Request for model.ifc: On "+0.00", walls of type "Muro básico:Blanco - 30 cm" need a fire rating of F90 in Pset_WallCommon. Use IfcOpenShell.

First a look at what the model holds.

```python
import ifcopenshell
import ifcopenshell.util.element

model = ifcopenshell.open("model.ifc")
print(model.schema)
storey = next(s for s in model.by_type("IfcBuildingStorey") if s.Name == "+0.00")
walls = [e for e in ifcopenshell.util.element.get_decomposition(storey) if e.is_a("IfcWall")]
seen = {}
for e in walls:
    element_type = ifcopenshell.util.element.get_type(e)
    key = (element_type.Name if element_type != e and element_type else None, ifcopenshell.util.element.get_pset(e, "Pset_WallCommon", "FireRating"))
    seen[key] = seen.get(key, 0) + 1
for (name, value), count in sorted(seen.items(), key=str):
    print(count, "x", name, "|", value)
```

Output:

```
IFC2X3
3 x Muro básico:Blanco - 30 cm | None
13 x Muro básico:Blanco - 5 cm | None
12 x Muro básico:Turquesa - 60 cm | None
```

```python
import ifcopenshell
import ifcopenshell.api.pset
import ifcopenshell.util.element

model = ifcopenshell.open("model.ifc")

storey = next(s for s in model.by_type("IfcBuildingStorey") if s.Name == "+0.00")
walls = [e for e in ifcopenshell.util.element.get_decomposition(storey) if e.is_a("IfcWall")]

count = 0
for e in walls:
    element_type = ifcopenshell.util.element.get_type(e)
    if element_type in (None, e) or element_type.Name != "Muro básico:Blanco - 30 cm":
        continue
    # add_pset returns the element's existing set when there is one.
    pset = ifcopenshell.api.pset.add_pset(model, product=e, name="Pset_WallCommon")
    ifcopenshell.api.pset.edit_pset(model, pset=pset, properties={"FireRating": "F90"})
    count += 1

print(count, "walls updated")

model.write("model_edited.ifc")
```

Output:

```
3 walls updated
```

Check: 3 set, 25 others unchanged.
